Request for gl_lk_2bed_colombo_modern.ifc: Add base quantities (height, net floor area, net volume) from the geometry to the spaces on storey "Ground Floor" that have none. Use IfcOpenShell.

First a look at what the model holds.

```python
import ifcopenshell
import ifcopenshell.util.element
import ifcopenshell.util.unit

model = ifcopenshell.open("gl_lk_2bed_colombo_modern.ifc")
print(model.schema)
for unit_type in ("LENGTHUNIT", "AREAUNIT", "VOLUMEUNIT"):
    print(unit_type, ifcopenshell.util.unit.calculate_unit_scale(model, unit_type))
storey = next(s for s in model.by_type("IfcBuildingStorey") if s.Name == "Ground Floor")
spaces = [e for e in ifcopenshell.util.element.get_decomposition(storey) if e.is_a("IfcSpace")]
for e in sorted(spaces, key=lambda e: e.id()):
    print(e.id(), e.is_a(), e.Name, list(ifcopenshell.util.element.get_psets(e, qtos_only=True)), sep=" | ")
```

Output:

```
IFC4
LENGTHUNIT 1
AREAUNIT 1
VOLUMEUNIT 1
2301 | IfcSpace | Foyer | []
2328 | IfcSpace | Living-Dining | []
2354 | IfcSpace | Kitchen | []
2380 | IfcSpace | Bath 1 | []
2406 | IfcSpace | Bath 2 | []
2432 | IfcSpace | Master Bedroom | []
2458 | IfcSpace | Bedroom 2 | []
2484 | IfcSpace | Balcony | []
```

```python
import ifcopenshell
import ifcopenshell.api.pset
import ifcopenshell.geom
import ifcopenshell.util.element
import ifcopenshell.util.shape
import ifcopenshell.util.unit

model = ifcopenshell.open("gl_lk_2bed_colombo_modern.ifc")
unit_scale = ifcopenshell.util.unit.calculate_unit_scale(model)
area_scale = ifcopenshell.util.unit.calculate_unit_scale(model, "AREAUNIT")
volume_scale = ifcopenshell.util.unit.calculate_unit_scale(model, "VOLUMEUNIT")
settings = ifcopenshell.geom.settings()

storey = next(s for s in model.by_type("IfcBuildingStorey") if s.Name == "Ground Floor")
spaces = [e for e in ifcopenshell.util.element.get_decomposition(storey) if e.is_a("IfcSpace")]

for e in sorted(spaces, key=lambda e: e.id()):
    if ifcopenshell.util.element.get_psets(e, qtos_only=True, should_inherit=False):
        continue
    # Geometry comes back in metres, in the element's own axes.
    shape = ifcopenshell.geom.create_shape(settings, e)
    values = {
        "Height": ifcopenshell.util.shape.get_z(shape.geometry) / unit_scale,
        "NetFloorArea": ifcopenshell.util.shape.get_footprint_area(shape.geometry) / area_scale,
        "NetVolume": ifcopenshell.util.shape.get_volume(shape.geometry) / volume_scale,
    }
    qto = ifcopenshell.api.pset.add_qto(model, product=e, name="Qto_SpaceBaseQuantities")
    ifcopenshell.api.pset.edit_qto(model, qto=qto, properties=values)
    print(e.id(), {k: round(v, 3) for k, v in values.items()})

model.write("gl_lk_2bed_colombo_modern_rev.ifc")
```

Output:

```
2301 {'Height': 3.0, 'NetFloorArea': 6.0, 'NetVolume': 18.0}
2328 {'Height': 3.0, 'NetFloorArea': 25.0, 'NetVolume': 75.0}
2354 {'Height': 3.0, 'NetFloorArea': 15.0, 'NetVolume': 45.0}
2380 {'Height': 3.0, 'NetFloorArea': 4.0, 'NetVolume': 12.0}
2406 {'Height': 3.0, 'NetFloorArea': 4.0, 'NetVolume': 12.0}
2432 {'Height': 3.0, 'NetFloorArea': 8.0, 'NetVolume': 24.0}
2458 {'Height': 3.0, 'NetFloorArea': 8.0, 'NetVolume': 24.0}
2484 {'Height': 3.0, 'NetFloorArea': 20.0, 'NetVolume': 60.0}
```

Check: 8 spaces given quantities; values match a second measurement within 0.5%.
